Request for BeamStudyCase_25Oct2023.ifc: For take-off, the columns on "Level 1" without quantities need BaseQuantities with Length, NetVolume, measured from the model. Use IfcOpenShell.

First a look at what the model holds.

```python
import ifcopenshell
import ifcopenshell.util.element
import ifcopenshell.util.unit

model = ifcopenshell.open("BeamStudyCase_25Oct2023.ifc")
print(model.schema)
for unit_type in ("LENGTHUNIT", "AREAUNIT", "VOLUMEUNIT"):
    print(unit_type, ifcopenshell.util.unit.calculate_unit_scale(model, unit_type))
storey = next(s for s in model.by_type("IfcBuildingStorey") if s.Name == "Level 1")
columns = [e for e in ifcopenshell.util.element.get_decomposition(storey) if e.is_a("IfcColumn")]
for e in sorted(columns, key=lambda e: e.id()):
    print(e.id(), e.is_a(), e.Name, list(ifcopenshell.util.element.get_psets(e, qtos_only=True)), sep=" | ")
```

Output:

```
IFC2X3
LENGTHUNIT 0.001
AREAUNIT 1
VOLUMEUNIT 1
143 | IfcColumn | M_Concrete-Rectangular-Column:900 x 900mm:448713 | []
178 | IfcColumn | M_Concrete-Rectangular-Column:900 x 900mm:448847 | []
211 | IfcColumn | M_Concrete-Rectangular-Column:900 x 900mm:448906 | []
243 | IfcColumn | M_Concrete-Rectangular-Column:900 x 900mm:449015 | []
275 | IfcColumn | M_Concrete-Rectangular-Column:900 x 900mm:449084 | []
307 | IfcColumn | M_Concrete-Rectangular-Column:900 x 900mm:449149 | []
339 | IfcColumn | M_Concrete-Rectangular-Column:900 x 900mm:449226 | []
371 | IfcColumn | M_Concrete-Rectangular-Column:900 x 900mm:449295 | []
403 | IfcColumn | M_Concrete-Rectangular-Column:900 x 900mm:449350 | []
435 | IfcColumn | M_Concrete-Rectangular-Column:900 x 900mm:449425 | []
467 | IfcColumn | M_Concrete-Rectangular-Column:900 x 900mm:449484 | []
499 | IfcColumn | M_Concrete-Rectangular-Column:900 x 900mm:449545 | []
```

```python
import ifcopenshell
import ifcopenshell.api.pset
import ifcopenshell.geom
import ifcopenshell.util.element
import ifcopenshell.util.shape
import ifcopenshell.util.unit

model = ifcopenshell.open("BeamStudyCase_25Oct2023.ifc")
unit_scale = ifcopenshell.util.unit.calculate_unit_scale(model)
volume_scale = ifcopenshell.util.unit.calculate_unit_scale(model, "VOLUMEUNIT")
settings = ifcopenshell.geom.settings()

storey = next(s for s in model.by_type("IfcBuildingStorey") if s.Name == "Level 1")
columns = [e for e in ifcopenshell.util.element.get_decomposition(storey) if e.is_a("IfcColumn")]

for e in sorted(columns, key=lambda e: e.id()):
    if ifcopenshell.util.element.get_psets(e, qtos_only=True, should_inherit=False):
        continue
    # Geometry comes back in metres, in the element's own axes.
    shape = ifcopenshell.geom.create_shape(settings, e)
    values = {
        "Length": ifcopenshell.util.shape.get_z(shape.geometry) / unit_scale,
        "NetVolume": ifcopenshell.util.shape.get_volume(shape.geometry) / volume_scale,
    }
    qto = ifcopenshell.api.pset.add_qto(model, product=e, name="BaseQuantities")
    ifcopenshell.api.pset.edit_qto(model, qto=qto, properties=values)
    print(e.id(), {k: round(v, 3) for k, v in values.items()})

model.write("BeamStudyCase_25Oct2023_v2.ifc")
```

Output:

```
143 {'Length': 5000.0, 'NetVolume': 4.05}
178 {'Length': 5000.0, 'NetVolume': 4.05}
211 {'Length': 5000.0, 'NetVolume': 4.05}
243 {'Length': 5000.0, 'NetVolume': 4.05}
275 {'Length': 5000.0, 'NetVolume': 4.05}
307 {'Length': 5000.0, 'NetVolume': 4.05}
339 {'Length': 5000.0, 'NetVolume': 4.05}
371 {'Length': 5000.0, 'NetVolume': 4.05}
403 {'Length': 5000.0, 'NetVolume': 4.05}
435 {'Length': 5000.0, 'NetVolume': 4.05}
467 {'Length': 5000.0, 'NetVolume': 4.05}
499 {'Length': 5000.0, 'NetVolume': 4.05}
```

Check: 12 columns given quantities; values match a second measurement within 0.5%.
